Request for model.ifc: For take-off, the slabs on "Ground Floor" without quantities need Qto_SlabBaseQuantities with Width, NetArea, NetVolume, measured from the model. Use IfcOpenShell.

First a look at what the model holds.

```python
import ifcopenshell
import ifcopenshell.util.element
import ifcopenshell.util.unit

model = ifcopenshell.open("model.ifc")
print(model.schema)
for unit_type in ("LENGTHUNIT", "AREAUNIT", "VOLUMEUNIT"):
    print(unit_type, ifcopenshell.util.unit.calculate_unit_scale(model, unit_type))
storey = next(s for s in model.by_type("IfcBuildingStorey") if s.Name == "Ground Floor")
slabs = [e for e in ifcopenshell.util.element.get_decomposition(storey) if e.is_a("IfcSlab")]
for e in sorted(slabs, key=lambda e: e.id()):
    print(e.id(), e.is_a(), e.Name, list(ifcopenshell.util.element.get_psets(e, qtos_only=True)), sep=" | ")
```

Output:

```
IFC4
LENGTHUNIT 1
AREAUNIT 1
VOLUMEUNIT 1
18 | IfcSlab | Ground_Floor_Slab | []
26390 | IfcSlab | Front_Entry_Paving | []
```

```python
import ifcopenshell
import ifcopenshell.api.pset
import ifcopenshell.geom
import ifcopenshell.util.element
import ifcopenshell.util.shape
import ifcopenshell.util.unit

model = ifcopenshell.open("model.ifc")
unit_scale = ifcopenshell.util.unit.calculate_unit_scale(model)
area_scale = ifcopenshell.util.unit.calculate_unit_scale(model, "AREAUNIT")
volume_scale = ifcopenshell.util.unit.calculate_unit_scale(model, "VOLUMEUNIT")
settings = ifcopenshell.geom.settings()

storey = next(s for s in model.by_type("IfcBuildingStorey") if s.Name == "Ground Floor")
slabs = [e for e in ifcopenshell.util.element.get_decomposition(storey) if e.is_a("IfcSlab")]

for e in sorted(slabs, key=lambda e: e.id()):
    if ifcopenshell.util.element.get_psets(e, qtos_only=True, should_inherit=False):
        continue
    # Geometry comes back in metres, in the element's own axes.
    shape = ifcopenshell.geom.create_shape(settings, e)
    values = {
        "Width": ifcopenshell.util.shape.get_z(shape.geometry) / unit_scale,
        "NetArea": ifcopenshell.util.shape.get_footprint_area(shape.geometry) / area_scale,
        "NetVolume": ifcopenshell.util.shape.get_volume(shape.geometry) / volume_scale,
    }
    qto = ifcopenshell.api.pset.add_qto(model, product=e, name="Qto_SlabBaseQuantities")
    ifcopenshell.api.pset.edit_qto(model, qto=qto, properties=values)
    print(e.id(), {k: round(v, 3) for k, v in values.items()})

model.write("model_updated.ifc")
```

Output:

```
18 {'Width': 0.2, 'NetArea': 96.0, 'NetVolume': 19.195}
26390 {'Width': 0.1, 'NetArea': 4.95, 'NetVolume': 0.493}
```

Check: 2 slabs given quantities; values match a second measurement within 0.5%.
